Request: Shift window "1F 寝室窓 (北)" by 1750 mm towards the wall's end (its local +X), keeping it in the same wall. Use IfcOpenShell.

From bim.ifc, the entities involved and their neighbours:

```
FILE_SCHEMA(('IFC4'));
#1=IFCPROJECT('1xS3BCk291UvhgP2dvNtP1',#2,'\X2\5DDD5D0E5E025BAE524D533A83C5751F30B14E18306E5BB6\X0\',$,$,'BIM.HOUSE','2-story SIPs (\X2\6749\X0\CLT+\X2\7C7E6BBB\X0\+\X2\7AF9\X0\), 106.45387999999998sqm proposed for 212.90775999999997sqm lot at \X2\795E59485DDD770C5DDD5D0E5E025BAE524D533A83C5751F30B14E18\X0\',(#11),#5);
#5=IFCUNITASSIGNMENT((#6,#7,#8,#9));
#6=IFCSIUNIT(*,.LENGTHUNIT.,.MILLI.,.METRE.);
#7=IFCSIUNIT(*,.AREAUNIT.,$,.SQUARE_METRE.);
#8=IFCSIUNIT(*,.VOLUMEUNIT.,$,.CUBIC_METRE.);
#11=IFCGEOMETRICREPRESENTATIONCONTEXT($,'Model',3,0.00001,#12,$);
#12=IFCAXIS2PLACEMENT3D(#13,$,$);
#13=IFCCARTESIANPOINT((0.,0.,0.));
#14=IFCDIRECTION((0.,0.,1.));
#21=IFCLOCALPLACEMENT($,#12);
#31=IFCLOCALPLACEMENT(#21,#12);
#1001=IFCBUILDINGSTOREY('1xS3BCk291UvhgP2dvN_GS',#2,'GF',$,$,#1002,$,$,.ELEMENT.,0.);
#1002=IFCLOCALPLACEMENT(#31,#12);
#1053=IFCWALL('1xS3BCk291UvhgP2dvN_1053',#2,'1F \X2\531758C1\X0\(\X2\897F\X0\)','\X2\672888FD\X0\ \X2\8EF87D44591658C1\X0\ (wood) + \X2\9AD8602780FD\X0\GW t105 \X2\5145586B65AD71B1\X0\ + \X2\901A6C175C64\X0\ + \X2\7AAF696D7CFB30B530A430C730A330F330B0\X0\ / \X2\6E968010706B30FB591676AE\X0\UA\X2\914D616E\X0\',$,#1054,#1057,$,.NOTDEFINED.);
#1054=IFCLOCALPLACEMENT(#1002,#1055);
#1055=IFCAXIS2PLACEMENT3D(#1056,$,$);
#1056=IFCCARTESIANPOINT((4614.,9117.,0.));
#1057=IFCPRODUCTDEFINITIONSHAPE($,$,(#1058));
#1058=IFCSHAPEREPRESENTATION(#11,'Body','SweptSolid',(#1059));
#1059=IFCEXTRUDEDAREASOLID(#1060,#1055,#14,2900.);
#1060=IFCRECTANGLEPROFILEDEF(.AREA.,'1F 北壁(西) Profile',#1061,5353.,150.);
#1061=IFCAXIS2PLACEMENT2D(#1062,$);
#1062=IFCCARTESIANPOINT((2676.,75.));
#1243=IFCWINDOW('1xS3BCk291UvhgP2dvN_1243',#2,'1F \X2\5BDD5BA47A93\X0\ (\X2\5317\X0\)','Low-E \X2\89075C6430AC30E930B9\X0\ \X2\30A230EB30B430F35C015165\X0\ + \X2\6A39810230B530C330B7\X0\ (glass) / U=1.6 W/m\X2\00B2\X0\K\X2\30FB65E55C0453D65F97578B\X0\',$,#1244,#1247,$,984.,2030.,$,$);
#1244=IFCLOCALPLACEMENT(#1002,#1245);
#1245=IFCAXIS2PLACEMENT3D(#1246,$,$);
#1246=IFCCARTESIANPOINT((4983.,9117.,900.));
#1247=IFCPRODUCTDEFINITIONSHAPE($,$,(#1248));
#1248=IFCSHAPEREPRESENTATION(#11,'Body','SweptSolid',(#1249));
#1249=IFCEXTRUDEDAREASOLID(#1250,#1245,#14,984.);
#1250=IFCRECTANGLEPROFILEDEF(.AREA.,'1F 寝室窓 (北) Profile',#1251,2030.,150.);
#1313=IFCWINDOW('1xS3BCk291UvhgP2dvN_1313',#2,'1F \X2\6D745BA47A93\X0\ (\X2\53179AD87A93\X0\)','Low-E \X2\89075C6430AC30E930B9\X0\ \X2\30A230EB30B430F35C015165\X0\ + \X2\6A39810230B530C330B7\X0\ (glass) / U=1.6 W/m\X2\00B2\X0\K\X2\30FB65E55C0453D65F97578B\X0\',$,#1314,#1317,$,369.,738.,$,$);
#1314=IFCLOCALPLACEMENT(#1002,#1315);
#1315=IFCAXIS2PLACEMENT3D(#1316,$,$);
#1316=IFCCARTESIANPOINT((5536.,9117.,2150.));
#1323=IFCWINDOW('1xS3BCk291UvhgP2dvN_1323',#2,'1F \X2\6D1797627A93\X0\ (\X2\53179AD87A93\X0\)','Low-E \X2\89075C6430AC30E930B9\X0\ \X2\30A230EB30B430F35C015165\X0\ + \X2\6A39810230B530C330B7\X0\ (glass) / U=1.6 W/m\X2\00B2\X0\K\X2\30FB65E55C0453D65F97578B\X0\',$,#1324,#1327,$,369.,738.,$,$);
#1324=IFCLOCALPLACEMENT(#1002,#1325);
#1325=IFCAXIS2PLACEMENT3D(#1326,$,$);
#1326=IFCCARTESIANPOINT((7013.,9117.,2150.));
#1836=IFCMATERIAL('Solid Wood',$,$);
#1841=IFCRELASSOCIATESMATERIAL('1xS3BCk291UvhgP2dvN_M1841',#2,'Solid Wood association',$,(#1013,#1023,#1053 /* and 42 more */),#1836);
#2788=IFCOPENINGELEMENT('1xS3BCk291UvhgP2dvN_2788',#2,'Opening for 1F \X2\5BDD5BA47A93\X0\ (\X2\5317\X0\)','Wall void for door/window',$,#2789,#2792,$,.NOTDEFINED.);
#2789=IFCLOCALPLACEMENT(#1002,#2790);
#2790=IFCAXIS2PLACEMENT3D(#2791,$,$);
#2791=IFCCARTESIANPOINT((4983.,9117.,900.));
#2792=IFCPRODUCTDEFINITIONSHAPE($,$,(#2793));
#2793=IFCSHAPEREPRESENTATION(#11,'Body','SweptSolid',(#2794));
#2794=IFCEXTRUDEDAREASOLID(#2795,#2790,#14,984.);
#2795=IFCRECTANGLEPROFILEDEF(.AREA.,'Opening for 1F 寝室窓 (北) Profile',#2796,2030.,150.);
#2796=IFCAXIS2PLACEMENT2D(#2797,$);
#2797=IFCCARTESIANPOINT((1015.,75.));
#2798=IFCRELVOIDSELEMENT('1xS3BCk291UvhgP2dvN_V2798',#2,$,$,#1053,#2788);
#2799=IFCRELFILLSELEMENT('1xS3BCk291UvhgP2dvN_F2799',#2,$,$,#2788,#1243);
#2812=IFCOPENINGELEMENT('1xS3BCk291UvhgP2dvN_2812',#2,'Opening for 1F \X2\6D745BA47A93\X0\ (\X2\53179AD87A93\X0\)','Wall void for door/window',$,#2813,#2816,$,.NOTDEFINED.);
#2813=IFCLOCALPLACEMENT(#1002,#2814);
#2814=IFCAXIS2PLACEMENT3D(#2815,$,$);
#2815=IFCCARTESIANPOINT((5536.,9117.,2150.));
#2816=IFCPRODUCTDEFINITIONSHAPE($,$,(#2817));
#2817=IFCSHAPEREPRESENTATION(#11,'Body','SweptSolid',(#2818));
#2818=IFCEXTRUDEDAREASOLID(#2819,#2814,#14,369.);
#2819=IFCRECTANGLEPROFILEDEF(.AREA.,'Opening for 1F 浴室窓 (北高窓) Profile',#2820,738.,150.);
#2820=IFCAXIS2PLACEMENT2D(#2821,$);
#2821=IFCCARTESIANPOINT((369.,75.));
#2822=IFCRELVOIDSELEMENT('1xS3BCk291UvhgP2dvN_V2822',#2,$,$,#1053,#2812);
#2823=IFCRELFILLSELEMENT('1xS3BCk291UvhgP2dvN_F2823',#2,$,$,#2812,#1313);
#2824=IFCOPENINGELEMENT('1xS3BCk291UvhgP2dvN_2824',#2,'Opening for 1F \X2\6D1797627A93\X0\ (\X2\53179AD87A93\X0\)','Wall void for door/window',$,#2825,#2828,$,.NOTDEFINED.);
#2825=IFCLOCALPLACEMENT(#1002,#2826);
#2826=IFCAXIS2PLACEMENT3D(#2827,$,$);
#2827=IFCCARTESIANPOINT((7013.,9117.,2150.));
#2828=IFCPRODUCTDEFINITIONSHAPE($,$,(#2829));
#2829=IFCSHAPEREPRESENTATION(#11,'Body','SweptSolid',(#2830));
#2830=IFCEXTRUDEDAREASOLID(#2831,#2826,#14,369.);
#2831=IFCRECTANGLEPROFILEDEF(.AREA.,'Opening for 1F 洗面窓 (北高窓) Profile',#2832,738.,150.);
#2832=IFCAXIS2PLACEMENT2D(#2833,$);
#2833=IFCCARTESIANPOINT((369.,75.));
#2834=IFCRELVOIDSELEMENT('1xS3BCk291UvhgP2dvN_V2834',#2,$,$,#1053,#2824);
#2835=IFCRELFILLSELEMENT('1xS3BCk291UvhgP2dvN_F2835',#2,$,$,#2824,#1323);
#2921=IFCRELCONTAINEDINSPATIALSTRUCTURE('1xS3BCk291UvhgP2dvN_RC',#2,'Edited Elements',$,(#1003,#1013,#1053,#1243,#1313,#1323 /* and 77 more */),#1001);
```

```python
import ifcopenshell
import ifcopenshell.api.geometry
import ifcopenshell.util.placement
import ifcopenshell.util.unit

model = ifcopenshell.open("bim.ifc")
unit_scale = ifcopenshell.util.unit.calculate_unit_scale(model)

window = model.by_guid("1xS3BCk291UvhgP2dvN_1243")
opening = window.FillsVoids[0].RelatingOpeningElement
wall = opening.VoidsElements[0].RelatingBuildingElement

wall_matrix = ifcopenshell.util.placement.get_local_placement(wall.ObjectPlacement)
shift = wall_matrix[:3, 0] * 1.75 / unit_scale
before = ifcopenshell.util.placement.get_local_placement(window.ObjectPlacement)[:3, 3].copy()

# The window is not placed relative to its opening, so move both.
for product in (opening, window):
    matrix = ifcopenshell.util.placement.get_local_placement(product.ObjectPlacement)
    matrix[:3, 3] += shift
    ifcopenshell.api.geometry.edit_object_placement(model, product=product, matrix=matrix, is_si=False)

after = ifcopenshell.util.placement.get_local_placement(window.ObjectPlacement)[:3, 3]
print("window moved by", (after - before).round(3) + 0.0)

model.write("bim_updated.ifc")
```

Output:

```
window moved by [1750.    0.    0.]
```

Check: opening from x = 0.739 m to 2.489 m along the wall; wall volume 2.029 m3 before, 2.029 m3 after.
